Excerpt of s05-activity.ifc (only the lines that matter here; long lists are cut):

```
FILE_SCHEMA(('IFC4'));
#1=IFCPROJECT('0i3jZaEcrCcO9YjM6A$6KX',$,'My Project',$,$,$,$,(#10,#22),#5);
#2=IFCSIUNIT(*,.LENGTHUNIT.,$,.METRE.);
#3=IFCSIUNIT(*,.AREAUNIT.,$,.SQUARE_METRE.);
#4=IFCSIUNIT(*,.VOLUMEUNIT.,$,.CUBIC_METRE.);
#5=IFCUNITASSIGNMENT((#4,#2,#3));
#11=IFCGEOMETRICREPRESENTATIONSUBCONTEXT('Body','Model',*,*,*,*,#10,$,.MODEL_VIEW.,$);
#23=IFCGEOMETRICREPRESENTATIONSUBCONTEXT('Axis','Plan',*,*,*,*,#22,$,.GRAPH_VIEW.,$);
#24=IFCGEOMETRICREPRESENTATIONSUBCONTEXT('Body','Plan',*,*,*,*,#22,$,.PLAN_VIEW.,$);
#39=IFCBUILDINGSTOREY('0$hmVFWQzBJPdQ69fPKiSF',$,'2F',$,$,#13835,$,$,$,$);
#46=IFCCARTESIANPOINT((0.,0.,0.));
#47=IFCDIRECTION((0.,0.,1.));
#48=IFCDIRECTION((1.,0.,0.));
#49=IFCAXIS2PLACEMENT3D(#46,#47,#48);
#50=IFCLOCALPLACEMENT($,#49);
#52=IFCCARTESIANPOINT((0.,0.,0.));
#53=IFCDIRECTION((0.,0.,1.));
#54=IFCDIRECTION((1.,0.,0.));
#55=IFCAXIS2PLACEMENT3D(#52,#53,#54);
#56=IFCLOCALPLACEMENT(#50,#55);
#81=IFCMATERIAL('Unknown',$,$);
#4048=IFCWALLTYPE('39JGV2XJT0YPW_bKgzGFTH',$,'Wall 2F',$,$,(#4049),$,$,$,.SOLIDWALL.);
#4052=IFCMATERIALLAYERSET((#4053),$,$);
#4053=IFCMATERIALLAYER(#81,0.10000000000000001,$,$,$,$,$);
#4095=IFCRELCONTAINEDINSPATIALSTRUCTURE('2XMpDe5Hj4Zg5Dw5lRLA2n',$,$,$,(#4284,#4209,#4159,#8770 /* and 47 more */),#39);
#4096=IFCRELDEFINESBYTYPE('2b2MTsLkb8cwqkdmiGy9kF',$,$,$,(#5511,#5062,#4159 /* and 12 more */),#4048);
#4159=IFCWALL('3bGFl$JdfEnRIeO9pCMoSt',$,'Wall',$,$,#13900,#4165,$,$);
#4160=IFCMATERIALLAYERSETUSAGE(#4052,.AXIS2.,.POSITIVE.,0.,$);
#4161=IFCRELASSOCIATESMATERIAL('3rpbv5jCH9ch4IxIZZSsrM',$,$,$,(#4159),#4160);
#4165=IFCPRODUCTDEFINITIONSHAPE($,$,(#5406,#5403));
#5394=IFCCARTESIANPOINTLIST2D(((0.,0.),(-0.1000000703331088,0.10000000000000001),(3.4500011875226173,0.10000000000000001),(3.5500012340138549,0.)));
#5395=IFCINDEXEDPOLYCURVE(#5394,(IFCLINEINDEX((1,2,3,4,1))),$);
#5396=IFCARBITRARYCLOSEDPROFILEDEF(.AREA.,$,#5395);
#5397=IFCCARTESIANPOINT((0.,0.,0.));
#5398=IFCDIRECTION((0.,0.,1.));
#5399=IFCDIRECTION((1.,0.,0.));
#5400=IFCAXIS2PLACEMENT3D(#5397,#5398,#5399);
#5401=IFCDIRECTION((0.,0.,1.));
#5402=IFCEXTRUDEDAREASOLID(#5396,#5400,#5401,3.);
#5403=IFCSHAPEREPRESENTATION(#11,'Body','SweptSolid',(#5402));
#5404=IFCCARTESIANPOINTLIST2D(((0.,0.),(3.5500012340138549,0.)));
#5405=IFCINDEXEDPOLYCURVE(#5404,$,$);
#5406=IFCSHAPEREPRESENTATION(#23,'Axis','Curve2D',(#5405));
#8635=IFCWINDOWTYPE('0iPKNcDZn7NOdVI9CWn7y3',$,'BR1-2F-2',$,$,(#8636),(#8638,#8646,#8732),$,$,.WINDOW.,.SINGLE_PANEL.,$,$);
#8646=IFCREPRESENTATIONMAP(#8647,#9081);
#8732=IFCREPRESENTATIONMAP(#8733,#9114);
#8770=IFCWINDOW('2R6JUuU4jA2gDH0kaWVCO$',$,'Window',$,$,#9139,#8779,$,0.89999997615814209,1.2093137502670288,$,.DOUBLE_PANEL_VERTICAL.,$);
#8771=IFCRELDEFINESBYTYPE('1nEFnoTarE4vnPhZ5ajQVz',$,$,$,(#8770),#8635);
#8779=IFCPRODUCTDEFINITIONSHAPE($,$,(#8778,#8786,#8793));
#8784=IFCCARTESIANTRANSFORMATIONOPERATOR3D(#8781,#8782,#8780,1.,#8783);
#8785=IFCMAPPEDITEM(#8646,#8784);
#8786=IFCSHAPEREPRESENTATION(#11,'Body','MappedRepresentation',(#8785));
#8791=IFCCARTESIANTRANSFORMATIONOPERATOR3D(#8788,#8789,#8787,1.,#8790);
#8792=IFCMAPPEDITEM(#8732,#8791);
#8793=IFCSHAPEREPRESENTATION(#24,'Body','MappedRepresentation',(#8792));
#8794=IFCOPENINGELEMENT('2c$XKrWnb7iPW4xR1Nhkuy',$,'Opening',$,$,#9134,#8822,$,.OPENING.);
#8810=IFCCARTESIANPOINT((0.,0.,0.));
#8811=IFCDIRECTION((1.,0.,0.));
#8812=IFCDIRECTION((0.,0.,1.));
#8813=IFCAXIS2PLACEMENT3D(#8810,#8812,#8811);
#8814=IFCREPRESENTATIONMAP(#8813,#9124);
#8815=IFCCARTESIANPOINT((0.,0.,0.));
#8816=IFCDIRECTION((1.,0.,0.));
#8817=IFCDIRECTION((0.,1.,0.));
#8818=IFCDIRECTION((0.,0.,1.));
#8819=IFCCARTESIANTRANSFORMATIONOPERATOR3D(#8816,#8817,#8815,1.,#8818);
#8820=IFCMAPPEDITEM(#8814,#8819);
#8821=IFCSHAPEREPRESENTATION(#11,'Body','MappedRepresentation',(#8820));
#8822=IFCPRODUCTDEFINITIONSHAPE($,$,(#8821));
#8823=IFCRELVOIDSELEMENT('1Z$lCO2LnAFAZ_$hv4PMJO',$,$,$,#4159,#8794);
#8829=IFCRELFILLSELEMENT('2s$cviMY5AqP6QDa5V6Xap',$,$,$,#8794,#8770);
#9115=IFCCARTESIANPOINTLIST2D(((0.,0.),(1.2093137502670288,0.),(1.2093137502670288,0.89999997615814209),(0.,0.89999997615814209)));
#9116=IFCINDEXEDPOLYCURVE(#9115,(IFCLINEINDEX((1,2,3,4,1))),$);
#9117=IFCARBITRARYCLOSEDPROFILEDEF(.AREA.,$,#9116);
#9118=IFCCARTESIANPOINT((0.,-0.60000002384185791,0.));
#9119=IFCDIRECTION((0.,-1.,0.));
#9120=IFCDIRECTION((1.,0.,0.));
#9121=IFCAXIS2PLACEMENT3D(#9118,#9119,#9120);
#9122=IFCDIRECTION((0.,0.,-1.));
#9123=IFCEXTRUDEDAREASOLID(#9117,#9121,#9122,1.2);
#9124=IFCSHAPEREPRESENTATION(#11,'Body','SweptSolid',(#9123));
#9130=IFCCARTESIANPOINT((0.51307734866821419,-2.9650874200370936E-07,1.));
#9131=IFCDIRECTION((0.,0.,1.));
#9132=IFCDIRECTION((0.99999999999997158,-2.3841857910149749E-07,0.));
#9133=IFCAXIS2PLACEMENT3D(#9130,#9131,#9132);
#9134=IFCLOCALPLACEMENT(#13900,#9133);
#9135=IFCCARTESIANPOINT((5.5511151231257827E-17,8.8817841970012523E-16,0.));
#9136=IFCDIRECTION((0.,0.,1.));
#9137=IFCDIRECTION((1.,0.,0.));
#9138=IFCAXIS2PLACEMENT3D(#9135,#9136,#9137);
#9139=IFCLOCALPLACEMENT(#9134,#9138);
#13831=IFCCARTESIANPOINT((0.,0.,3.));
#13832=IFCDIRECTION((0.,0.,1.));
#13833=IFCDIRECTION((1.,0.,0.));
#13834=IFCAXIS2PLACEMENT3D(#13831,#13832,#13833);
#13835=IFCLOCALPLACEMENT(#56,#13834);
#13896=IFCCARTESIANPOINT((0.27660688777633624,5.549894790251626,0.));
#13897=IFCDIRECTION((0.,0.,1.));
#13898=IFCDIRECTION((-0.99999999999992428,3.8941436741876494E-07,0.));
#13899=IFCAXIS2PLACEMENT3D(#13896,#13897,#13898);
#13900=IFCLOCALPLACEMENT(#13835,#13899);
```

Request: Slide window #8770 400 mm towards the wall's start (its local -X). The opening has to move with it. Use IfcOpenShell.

```python
import ifcopenshell
import ifcopenshell.api.geometry
import ifcopenshell.util.placement

model = ifcopenshell.open("s05-activity.ifc")

window = model.by_guid("2R6JUuU4jA2gDH0kaWVCO$")
opening = window.FillsVoids[0].RelatingOpeningElement
wall = opening.VoidsElements[0].RelatingBuildingElement

wall_matrix = ifcopenshell.util.placement.get_local_placement(wall.ObjectPlacement)
shift = wall_matrix[:3, 0] * -0.4
before = ifcopenshell.util.placement.get_local_placement(window.ObjectPlacement)[:3, 3].copy()

# The window is placed relative to its opening, so it follows when the opening moves.
matrix = ifcopenshell.util.placement.get_local_placement(opening.ObjectPlacement)
matrix[:3, 3] += shift
ifcopenshell.api.geometry.edit_object_placement(
    model, product=opening, matrix=matrix, is_si=False, should_transform_children=True
)

after = ifcopenshell.util.placement.get_local_placement(window.ObjectPlacement)[:3, 3]
print("window moved by", (after - before).round(3) + 0.0)

model.write("s05-activity_updated.ifc")
```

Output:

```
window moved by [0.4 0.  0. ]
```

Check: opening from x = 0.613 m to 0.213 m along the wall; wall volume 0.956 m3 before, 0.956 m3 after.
